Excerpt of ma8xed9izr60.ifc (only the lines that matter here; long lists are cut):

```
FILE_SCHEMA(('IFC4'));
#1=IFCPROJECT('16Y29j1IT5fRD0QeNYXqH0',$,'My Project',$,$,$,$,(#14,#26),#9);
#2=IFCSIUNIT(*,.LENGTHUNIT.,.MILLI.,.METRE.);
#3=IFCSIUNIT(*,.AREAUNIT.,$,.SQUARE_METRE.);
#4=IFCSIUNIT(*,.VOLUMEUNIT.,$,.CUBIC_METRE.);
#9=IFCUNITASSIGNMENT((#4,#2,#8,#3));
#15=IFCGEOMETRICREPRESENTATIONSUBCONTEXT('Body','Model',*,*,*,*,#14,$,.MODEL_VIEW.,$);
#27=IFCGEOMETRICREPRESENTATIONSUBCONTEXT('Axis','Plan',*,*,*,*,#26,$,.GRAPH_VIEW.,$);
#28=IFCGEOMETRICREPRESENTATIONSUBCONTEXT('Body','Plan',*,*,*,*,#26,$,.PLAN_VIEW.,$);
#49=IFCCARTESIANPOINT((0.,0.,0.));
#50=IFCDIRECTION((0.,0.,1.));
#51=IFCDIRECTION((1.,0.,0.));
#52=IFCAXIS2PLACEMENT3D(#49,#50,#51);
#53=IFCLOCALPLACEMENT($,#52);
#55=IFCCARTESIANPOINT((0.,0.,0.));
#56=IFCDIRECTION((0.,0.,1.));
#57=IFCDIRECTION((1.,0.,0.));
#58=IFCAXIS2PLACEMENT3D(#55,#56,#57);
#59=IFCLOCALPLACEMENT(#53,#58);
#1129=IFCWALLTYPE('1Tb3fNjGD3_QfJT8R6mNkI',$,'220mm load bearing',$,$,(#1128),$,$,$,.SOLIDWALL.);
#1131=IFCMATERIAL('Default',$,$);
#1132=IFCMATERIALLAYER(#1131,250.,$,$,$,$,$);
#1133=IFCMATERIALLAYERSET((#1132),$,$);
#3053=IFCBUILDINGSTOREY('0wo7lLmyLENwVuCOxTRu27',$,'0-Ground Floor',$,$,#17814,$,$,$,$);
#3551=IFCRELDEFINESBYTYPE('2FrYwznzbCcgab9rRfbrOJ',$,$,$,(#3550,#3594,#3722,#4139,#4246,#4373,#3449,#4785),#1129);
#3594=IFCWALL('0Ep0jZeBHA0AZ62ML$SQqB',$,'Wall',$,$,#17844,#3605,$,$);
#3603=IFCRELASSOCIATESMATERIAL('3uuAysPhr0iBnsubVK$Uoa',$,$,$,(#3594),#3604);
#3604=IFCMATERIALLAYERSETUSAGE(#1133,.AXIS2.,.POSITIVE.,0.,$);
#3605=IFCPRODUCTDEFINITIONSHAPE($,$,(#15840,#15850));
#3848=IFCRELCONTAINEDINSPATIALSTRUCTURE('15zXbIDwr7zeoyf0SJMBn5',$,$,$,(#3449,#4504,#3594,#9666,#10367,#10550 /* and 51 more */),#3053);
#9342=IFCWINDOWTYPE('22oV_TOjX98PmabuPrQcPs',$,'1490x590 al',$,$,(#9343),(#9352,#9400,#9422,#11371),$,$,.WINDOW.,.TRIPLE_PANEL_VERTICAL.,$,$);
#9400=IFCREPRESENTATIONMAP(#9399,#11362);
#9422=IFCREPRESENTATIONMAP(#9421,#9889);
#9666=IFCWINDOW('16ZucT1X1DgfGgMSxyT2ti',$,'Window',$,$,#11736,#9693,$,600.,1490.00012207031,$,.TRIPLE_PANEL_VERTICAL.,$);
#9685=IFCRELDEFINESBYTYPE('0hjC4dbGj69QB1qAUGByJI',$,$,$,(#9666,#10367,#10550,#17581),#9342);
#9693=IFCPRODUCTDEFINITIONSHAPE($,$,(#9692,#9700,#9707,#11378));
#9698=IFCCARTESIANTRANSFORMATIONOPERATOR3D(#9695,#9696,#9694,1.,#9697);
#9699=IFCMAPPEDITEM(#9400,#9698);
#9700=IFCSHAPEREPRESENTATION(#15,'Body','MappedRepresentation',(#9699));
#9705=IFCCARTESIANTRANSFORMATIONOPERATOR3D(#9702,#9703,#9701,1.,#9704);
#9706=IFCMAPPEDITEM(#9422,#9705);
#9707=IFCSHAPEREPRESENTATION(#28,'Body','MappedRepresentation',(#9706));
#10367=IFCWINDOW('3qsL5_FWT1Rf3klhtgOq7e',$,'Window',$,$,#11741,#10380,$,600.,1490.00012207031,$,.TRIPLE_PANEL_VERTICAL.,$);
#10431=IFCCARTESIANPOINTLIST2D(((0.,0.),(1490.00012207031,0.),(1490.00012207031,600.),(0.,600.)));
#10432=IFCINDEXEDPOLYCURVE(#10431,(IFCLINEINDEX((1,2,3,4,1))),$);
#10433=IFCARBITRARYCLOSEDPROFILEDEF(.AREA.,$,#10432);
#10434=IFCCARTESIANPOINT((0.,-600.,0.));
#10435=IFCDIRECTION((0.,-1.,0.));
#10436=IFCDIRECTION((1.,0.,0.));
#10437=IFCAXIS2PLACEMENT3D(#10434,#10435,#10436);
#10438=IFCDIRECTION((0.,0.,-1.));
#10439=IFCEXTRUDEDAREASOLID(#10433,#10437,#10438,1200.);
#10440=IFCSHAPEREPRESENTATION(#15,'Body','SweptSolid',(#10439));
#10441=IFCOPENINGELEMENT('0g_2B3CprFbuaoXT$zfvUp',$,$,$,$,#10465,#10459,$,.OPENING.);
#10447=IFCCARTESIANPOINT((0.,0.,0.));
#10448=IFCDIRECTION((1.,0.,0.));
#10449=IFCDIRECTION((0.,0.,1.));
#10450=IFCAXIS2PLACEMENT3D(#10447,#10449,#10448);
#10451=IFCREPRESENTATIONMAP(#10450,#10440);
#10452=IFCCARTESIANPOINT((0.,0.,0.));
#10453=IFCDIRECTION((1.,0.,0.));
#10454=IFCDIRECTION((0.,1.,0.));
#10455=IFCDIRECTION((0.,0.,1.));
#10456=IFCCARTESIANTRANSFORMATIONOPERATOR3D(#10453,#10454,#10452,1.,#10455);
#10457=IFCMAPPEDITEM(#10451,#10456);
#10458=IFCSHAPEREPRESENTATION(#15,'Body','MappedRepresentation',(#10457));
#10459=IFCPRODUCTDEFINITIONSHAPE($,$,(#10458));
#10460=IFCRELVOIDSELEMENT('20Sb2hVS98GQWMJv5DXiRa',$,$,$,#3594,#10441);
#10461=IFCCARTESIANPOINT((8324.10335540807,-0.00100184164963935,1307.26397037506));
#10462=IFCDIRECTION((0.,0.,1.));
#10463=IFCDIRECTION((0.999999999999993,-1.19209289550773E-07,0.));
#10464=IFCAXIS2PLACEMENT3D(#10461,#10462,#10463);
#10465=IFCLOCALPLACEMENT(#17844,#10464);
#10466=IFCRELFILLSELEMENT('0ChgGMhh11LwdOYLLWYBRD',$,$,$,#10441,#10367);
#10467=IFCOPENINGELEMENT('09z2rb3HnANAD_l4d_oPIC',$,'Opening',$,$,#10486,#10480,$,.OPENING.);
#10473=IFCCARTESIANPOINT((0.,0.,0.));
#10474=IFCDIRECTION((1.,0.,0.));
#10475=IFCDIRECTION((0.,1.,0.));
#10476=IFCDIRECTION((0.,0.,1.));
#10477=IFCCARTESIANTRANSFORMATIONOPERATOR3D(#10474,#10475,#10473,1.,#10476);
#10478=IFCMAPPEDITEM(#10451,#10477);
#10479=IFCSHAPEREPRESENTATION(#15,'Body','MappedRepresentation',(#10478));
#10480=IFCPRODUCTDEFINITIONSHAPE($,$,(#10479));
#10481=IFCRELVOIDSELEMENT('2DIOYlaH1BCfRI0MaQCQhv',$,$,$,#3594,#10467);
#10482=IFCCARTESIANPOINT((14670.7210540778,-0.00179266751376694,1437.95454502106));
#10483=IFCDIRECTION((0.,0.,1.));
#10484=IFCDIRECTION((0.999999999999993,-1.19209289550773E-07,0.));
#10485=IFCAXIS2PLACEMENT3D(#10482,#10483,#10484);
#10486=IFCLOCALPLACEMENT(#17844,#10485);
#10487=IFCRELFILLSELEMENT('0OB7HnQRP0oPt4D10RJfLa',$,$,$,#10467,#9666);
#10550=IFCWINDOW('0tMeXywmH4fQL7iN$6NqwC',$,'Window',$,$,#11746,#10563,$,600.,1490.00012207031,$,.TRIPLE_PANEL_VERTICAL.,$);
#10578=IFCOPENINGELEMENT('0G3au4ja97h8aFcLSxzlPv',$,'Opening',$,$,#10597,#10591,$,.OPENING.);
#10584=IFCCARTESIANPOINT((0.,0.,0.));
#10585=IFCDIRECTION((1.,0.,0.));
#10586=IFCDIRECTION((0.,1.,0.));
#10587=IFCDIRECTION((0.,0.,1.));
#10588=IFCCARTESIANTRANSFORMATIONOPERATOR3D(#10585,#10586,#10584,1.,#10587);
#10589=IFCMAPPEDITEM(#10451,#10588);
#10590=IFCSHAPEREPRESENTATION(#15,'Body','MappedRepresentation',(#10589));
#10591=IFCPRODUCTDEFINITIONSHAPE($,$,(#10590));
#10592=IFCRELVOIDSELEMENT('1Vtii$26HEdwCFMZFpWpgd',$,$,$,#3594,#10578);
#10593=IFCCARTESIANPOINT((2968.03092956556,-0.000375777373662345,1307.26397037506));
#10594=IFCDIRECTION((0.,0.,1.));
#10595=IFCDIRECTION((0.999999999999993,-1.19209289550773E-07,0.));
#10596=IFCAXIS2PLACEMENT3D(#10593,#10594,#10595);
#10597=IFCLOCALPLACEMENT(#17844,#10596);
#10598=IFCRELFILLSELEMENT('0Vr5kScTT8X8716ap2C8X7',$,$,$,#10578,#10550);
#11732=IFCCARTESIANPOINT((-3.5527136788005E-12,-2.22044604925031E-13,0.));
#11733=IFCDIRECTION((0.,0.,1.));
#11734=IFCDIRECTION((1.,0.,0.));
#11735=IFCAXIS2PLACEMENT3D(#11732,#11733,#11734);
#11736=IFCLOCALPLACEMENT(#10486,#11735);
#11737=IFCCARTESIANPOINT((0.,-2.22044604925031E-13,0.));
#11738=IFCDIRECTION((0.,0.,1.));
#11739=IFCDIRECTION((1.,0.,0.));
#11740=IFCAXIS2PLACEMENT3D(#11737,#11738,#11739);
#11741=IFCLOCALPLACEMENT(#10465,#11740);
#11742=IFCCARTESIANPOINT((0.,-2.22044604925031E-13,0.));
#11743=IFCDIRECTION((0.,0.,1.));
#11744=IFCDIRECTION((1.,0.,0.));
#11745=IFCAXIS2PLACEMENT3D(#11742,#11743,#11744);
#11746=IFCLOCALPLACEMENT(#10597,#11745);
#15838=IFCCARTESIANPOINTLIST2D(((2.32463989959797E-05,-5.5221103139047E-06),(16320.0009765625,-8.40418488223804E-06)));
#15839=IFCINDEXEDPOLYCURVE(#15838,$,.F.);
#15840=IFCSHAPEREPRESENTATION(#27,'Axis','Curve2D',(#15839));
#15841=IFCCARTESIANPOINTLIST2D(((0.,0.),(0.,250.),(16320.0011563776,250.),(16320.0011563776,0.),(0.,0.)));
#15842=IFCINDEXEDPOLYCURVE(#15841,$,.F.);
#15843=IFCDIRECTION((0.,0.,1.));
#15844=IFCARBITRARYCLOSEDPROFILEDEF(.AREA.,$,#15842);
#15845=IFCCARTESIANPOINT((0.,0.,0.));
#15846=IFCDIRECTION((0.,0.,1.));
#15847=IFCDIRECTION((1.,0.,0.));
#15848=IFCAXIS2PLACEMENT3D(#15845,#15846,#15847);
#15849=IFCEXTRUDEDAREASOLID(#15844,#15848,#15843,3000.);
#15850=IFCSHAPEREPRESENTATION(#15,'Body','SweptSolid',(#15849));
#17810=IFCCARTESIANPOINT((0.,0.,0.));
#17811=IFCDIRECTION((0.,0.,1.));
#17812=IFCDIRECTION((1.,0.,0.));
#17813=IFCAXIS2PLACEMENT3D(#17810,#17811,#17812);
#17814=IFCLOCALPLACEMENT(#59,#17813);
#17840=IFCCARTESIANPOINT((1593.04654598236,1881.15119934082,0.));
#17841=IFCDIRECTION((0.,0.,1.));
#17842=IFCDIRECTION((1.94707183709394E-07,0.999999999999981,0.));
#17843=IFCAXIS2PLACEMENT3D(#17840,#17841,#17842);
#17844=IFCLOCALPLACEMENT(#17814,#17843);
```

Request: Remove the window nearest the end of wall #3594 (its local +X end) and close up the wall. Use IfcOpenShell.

```python
import ifcopenshell
import ifcopenshell.api.feature
import ifcopenshell.api.root
import ifcopenshell.geom
import ifcopenshell.util.shape

model = ifcopenshell.open("ma8xed9izr60.ifc")
settings = ifcopenshell.geom.settings()


def volume(element):
    """Net volume in cubic metres, openings subtracted."""
    shape = ifcopenshell.geom.create_shape(settings, element)
    return ifcopenshell.util.shape.get_volume(shape.geometry)


window = model.by_guid("16ZucT1X1DgfGgMSxyT2ti")
opening = window.FillsVoids[0].RelatingOpeningElement
wall = opening.VoidsElements[0].RelatingBuildingElement
before = volume(wall)

ifcopenshell.api.root.remove_product(model, product=window)
ifcopenshell.api.feature.remove_feature(model, feature=opening)

after = volume(wall)

print(f"wall volume {before:.3f} -> {after:.3f} m3")

model.write("ma8xed9izr60_rev.ifc")
```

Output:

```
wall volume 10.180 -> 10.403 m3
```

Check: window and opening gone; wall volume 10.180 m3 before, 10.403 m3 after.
